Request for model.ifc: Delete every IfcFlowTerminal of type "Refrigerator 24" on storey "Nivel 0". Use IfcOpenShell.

First a look at what the model holds.

```python
import ifcopenshell
import ifcopenshell.util.element

model = ifcopenshell.open("model.ifc")
print(model.schema)
storey = next(s for s in model.by_type("IfcBuildingStorey") if s.Name == "Nivel 0")
terminals = [e for e in ifcopenshell.util.element.get_decomposition(storey) if e.is_a("IfcFlowTerminal")]
seen = {}
for e in terminals:
    element_type = ifcopenshell.util.element.get_type(e)
    name = element_type.Name if element_type not in (None, e) else None
    seen[name] = seen.get(name, 0) + 1
for name, count in sorted(seen.items(), key=str):
    print(count, "x", name)
```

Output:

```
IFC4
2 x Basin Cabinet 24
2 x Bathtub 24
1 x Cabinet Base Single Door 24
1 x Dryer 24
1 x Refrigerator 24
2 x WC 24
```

```python
import ifcopenshell
import ifcopenshell.api.root
import ifcopenshell.util.element

model = ifcopenshell.open("model.ifc")

storey = next(s for s in model.by_type("IfcBuildingStorey") if s.Name == "Nivel 0")
terminals = [e for e in ifcopenshell.util.element.get_decomposition(storey) if e.is_a("IfcFlowTerminal")]
targets = [e for e in terminals if (t := ifcopenshell.util.element.get_type(e)) not in (None, e) and t.Name == "Refrigerator 24"]

for e in targets:
    ifcopenshell.api.root.remove_product(model, product=e)
print(len(targets), "removed")

model.write("model_edited.ifc")
```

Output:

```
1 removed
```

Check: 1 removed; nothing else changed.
